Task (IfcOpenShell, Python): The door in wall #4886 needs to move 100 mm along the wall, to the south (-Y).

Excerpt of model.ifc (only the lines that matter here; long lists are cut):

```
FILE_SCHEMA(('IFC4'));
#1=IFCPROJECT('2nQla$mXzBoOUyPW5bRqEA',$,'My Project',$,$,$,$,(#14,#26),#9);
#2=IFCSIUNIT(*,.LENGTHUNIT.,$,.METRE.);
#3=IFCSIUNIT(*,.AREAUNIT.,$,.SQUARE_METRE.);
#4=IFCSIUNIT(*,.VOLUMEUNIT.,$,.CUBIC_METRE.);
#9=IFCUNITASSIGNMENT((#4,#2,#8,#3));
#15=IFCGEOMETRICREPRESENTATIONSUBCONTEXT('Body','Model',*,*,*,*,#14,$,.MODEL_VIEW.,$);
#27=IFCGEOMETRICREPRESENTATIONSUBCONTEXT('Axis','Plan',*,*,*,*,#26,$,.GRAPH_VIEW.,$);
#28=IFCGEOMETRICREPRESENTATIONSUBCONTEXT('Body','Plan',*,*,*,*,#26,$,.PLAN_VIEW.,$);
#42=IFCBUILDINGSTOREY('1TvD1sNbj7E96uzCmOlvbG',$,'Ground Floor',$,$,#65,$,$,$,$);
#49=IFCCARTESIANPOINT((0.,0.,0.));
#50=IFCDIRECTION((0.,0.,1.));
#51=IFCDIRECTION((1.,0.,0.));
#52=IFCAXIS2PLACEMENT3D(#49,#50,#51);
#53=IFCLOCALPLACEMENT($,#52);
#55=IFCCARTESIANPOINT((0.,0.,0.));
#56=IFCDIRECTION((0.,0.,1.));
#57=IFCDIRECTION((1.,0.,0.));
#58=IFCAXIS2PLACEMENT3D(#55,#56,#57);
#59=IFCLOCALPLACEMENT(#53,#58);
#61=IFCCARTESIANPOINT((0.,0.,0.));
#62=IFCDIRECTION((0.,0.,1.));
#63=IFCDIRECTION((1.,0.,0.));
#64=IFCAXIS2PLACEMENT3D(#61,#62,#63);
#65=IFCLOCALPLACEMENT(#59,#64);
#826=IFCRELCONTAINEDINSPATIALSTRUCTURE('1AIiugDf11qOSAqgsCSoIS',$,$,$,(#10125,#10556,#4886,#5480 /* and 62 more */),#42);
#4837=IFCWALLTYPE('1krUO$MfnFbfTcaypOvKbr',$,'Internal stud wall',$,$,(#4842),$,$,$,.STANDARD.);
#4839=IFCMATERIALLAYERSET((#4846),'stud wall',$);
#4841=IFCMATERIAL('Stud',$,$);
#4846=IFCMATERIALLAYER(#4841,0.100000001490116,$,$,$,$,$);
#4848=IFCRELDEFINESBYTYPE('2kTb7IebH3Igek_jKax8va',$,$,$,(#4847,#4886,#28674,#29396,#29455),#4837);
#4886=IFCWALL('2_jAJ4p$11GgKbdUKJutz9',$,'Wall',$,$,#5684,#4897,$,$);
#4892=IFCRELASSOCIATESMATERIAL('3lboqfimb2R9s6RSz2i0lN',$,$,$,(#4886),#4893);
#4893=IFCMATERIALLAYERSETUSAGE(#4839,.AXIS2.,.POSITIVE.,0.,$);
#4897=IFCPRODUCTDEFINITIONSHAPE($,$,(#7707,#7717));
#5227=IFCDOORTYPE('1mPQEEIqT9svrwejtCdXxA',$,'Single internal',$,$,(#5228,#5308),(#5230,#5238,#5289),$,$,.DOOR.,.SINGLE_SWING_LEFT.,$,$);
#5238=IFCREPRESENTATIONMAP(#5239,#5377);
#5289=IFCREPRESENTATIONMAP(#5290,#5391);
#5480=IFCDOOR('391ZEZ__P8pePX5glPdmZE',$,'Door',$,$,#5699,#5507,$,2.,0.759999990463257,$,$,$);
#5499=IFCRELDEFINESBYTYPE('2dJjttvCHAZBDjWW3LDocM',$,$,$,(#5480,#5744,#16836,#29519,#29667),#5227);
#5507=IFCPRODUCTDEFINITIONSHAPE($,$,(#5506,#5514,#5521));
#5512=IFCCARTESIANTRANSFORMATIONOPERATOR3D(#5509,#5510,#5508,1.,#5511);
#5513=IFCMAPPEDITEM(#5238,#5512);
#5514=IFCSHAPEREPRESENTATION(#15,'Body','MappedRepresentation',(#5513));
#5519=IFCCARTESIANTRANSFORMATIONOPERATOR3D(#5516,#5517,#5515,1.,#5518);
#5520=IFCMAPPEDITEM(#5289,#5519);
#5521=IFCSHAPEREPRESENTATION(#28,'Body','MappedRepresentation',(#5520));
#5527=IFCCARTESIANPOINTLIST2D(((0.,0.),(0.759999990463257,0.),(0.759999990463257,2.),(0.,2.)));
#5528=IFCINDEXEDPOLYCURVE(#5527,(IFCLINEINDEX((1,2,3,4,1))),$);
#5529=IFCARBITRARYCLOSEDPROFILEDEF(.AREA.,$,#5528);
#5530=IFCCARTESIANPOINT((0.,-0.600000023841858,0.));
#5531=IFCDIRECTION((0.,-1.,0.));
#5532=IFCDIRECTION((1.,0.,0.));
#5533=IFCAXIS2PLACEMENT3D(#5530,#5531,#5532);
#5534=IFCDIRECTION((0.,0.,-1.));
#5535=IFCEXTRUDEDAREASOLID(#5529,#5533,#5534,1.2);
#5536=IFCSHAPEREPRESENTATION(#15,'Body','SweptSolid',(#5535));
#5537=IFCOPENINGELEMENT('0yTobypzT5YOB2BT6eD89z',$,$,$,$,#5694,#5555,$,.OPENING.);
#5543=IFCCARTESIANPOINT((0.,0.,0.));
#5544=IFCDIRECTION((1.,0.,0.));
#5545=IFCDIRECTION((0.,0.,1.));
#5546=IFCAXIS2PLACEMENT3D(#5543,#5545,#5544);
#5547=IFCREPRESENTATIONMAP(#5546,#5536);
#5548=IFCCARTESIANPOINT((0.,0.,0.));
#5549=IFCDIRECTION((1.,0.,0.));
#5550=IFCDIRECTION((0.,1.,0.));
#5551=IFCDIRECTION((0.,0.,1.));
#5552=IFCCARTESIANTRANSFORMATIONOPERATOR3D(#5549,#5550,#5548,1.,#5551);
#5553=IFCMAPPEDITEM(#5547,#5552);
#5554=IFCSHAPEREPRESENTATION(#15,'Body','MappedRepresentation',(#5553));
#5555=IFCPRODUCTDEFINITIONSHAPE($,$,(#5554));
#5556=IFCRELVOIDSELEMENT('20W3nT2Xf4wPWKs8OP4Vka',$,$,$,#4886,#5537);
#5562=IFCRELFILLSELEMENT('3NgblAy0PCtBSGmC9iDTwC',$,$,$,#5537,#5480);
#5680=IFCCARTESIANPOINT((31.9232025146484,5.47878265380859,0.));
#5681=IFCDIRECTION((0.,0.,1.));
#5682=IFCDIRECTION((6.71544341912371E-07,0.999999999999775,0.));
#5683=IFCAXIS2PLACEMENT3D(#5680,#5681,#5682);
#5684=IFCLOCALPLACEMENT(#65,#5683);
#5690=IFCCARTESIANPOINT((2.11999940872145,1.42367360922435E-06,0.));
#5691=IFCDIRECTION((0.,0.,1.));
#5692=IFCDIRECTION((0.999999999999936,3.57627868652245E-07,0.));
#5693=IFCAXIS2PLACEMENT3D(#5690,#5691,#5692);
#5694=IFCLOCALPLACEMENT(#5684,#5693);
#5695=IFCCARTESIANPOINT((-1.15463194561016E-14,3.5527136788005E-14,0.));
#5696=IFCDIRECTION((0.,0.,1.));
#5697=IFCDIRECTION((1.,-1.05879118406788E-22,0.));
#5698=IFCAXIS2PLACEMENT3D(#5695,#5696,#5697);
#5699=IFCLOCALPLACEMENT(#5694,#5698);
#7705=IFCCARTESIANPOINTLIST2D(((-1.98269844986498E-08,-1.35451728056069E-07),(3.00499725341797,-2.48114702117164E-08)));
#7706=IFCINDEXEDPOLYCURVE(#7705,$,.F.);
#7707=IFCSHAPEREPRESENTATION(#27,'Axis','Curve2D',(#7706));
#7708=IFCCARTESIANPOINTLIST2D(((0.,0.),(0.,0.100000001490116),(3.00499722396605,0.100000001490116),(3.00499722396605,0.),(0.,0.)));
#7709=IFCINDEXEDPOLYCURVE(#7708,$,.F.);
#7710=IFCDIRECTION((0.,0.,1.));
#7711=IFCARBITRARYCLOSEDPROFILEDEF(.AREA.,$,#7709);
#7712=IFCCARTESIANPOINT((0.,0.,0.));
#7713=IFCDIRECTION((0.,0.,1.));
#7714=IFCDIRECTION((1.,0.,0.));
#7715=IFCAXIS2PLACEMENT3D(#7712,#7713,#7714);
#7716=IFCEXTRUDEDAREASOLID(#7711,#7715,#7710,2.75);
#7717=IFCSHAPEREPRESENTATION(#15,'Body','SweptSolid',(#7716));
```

```python
import ifcopenshell
import ifcopenshell.api.geometry
import ifcopenshell.util.placement
import ifcopenshell.util.unit

model = ifcopenshell.open("model.ifc")
unit_scale = ifcopenshell.util.unit.calculate_unit_scale(model)

door = model.by_id(5480)
opening = door.FillsVoids[0].RelatingOpeningElement
wall = opening.VoidsElements[0].RelatingBuildingElement

wall_matrix = ifcopenshell.util.placement.get_local_placement(wall.ObjectPlacement)
shift = wall_matrix[:3, 0] * -0.1 / unit_scale
before = ifcopenshell.util.placement.get_local_placement(door.ObjectPlacement)[:3, 3].copy()

# The door is placed relative to its opening, so it follows when the opening moves.
matrix = ifcopenshell.util.placement.get_local_placement(opening.ObjectPlacement)
matrix[:3, 3] += shift
ifcopenshell.api.geometry.edit_object_placement(
    model, product=opening, matrix=matrix, is_si=False, should_transform_children=True
)

after = ifcopenshell.util.placement.get_local_placement(door.ObjectPlacement)[:3, 3]
print("door moved by", (after - before).round(3) + 0.0)

model.write("model_rev.ifc")
```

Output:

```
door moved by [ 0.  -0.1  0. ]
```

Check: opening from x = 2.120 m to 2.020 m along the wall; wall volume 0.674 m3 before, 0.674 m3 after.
